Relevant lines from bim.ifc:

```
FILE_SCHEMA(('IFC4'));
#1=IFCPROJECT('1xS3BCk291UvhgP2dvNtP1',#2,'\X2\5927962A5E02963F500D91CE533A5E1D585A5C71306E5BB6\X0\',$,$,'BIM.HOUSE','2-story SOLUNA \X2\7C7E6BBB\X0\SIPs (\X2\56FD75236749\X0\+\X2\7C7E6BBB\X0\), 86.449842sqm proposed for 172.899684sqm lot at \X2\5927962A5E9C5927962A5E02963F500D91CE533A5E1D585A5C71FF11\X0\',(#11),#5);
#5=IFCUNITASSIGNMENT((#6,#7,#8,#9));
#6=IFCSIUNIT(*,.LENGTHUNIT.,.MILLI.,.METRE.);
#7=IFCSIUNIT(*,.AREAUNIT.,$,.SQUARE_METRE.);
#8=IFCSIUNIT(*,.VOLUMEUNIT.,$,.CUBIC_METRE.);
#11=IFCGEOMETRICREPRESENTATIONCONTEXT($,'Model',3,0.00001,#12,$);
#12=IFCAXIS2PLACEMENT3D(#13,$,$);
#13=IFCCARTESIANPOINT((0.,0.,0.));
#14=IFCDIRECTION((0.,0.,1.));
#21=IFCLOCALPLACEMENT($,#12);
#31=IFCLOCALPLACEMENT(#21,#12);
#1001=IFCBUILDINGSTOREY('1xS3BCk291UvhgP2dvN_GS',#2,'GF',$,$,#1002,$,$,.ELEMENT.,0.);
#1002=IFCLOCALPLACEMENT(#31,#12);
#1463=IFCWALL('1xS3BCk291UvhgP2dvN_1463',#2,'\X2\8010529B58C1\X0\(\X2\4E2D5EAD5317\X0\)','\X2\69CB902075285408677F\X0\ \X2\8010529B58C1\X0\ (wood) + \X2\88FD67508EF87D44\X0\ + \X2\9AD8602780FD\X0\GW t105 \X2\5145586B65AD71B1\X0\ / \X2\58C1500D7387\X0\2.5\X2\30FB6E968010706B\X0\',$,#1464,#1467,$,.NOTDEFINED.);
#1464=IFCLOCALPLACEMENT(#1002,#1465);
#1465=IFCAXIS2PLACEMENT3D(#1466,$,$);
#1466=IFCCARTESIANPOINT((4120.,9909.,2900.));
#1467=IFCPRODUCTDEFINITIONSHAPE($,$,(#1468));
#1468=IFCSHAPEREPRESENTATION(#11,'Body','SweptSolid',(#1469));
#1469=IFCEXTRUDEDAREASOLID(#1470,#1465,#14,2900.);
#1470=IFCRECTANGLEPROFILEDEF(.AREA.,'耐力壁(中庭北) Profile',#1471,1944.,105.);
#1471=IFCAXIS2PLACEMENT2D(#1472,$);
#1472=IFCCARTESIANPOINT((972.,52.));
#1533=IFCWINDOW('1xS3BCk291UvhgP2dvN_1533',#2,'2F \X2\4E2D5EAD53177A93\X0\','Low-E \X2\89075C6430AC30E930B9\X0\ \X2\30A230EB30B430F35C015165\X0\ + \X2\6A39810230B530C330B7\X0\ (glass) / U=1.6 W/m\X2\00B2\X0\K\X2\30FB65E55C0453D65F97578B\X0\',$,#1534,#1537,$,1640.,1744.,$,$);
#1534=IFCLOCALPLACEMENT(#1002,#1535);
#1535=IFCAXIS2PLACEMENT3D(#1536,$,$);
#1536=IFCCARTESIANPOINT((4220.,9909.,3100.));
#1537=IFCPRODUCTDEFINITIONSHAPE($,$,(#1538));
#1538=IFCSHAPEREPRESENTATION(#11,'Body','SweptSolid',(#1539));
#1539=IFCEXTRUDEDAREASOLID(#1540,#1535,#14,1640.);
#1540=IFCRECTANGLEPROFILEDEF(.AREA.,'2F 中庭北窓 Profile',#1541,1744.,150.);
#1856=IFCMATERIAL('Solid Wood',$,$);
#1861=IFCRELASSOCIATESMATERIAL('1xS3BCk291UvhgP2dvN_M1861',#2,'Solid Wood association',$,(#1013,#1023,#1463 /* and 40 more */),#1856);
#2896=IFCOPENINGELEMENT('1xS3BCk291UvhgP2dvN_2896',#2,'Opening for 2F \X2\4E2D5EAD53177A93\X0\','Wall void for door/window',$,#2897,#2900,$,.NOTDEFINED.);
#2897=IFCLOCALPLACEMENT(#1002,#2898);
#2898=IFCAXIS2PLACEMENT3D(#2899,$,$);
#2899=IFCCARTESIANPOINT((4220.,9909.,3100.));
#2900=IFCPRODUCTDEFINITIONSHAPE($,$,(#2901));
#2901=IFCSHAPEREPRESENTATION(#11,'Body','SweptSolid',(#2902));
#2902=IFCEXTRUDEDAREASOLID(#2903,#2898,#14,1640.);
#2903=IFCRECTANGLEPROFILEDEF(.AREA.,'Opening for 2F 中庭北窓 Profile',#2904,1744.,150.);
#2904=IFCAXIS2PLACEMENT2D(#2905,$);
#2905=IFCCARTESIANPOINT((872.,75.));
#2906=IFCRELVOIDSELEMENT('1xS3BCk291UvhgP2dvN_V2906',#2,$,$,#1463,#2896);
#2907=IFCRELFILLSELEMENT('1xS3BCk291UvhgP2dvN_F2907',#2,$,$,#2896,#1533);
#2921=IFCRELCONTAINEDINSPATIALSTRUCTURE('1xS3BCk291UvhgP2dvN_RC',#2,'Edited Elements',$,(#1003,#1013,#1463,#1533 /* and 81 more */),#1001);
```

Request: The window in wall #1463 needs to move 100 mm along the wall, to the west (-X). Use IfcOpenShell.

```python
import ifcopenshell
import ifcopenshell.api.geometry
import ifcopenshell.util.placement
import ifcopenshell.util.unit

model = ifcopenshell.open("bim.ifc")
unit_scale = ifcopenshell.util.unit.calculate_unit_scale(model)

window = model.by_id(1533)
opening = window.FillsVoids[0].RelatingOpeningElement
wall = opening.VoidsElements[0].RelatingBuildingElement

wall_matrix = ifcopenshell.util.placement.get_local_placement(wall.ObjectPlacement)
shift = wall_matrix[:3, 0] * -0.1 / unit_scale
before = ifcopenshell.util.placement.get_local_placement(window.ObjectPlacement)[:3, 3].copy()

# The window is not placed relative to its opening, so move both.
for product in (opening, window):
    matrix = ifcopenshell.util.placement.get_local_placement(product.ObjectPlacement)
    matrix[:3, 3] += shift
    ifcopenshell.api.geometry.edit_object_placement(model, product=product, matrix=matrix, is_si=False)

after = ifcopenshell.util.placement.get_local_placement(window.ObjectPlacement)[:3, 3]
print("window moved by", (after - before).round(3) + 0.0)

model.write("bim_edited.ifc")
```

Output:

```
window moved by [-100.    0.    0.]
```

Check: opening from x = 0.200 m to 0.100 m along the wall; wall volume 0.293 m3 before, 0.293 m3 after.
